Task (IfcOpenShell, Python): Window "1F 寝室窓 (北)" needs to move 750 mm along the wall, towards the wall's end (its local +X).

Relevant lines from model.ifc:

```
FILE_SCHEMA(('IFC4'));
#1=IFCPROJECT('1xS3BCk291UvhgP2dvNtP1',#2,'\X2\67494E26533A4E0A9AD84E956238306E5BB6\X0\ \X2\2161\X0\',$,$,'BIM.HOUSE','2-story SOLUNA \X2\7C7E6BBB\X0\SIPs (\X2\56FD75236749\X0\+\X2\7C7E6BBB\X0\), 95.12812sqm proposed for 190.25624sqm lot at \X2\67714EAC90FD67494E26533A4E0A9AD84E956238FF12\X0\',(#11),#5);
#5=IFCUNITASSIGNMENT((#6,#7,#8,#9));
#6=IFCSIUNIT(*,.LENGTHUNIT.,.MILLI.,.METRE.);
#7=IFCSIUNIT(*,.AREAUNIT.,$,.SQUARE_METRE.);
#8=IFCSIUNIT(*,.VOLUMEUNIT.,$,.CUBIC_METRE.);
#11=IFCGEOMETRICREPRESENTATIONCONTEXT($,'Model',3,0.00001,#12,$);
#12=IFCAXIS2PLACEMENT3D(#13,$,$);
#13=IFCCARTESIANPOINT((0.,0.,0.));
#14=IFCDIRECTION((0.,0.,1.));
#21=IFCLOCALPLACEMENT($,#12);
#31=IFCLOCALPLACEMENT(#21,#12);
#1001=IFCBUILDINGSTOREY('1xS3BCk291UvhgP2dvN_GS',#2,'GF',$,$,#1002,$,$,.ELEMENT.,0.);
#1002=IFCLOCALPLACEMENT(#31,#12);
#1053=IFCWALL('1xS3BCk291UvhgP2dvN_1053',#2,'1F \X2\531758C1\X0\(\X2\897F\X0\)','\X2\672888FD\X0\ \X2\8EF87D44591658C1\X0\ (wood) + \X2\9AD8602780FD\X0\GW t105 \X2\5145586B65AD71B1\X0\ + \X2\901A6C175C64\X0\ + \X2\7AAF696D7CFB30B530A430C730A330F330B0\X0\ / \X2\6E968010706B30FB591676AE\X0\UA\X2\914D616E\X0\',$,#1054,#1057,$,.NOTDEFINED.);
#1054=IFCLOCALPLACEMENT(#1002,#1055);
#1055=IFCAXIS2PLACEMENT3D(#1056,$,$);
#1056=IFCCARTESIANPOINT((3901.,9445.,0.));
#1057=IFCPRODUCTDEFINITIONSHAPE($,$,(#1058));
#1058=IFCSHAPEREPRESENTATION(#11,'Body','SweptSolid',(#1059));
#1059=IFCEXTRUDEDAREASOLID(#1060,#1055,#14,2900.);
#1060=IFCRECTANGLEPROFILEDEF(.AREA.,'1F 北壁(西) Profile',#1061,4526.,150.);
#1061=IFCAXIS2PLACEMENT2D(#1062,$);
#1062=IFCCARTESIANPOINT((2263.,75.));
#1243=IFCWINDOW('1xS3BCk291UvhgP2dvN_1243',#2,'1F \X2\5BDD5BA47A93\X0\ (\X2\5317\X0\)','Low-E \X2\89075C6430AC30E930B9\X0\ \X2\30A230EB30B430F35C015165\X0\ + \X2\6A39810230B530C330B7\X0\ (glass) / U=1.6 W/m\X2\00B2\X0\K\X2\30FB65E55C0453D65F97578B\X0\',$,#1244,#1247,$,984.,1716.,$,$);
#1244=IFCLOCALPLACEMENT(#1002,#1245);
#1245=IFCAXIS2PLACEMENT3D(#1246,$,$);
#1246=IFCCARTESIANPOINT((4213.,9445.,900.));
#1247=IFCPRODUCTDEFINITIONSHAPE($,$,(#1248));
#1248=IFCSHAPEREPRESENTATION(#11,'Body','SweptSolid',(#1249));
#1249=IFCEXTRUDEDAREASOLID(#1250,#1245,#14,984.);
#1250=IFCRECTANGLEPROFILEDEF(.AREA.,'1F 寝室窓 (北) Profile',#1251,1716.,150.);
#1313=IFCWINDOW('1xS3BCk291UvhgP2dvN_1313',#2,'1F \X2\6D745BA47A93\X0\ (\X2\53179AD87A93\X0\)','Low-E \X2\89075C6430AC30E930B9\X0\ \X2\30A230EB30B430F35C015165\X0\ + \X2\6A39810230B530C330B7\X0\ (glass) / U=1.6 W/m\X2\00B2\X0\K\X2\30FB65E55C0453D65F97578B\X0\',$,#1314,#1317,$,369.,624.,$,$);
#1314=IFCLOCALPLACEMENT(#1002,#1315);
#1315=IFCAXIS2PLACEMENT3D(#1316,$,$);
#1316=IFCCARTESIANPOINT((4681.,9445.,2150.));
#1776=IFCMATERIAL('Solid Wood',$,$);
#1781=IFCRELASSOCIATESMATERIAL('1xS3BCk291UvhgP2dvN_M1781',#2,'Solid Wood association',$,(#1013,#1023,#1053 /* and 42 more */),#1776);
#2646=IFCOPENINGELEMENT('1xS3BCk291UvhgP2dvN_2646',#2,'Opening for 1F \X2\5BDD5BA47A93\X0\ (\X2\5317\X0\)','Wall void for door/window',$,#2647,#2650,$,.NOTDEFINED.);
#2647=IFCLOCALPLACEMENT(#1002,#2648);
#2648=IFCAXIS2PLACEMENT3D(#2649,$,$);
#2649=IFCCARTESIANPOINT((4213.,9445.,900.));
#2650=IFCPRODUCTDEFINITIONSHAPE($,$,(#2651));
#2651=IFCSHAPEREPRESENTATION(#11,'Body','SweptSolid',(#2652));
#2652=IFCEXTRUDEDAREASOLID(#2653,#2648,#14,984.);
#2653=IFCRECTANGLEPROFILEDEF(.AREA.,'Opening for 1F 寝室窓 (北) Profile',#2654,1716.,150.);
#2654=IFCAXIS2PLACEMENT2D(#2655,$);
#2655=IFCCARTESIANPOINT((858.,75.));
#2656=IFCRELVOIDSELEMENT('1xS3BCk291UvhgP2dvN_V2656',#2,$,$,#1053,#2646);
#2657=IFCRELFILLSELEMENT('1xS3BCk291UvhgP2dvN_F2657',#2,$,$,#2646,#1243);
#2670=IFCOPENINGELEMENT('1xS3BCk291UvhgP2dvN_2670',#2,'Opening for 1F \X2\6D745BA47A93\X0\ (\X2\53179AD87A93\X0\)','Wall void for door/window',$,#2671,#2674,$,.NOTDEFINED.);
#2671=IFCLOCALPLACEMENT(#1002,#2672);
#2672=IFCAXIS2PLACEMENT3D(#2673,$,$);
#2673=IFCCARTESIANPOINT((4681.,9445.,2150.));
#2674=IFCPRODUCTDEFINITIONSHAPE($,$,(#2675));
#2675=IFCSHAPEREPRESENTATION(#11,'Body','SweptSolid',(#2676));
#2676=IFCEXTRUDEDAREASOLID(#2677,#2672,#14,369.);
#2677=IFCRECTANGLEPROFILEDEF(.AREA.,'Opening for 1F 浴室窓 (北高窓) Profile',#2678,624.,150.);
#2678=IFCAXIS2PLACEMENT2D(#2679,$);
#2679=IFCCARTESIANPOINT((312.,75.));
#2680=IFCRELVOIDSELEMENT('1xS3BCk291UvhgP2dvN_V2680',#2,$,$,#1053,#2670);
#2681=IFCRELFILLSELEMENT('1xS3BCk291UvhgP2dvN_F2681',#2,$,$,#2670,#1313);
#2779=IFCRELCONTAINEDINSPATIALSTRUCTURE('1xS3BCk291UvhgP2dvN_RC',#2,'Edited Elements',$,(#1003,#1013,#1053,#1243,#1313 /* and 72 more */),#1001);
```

```python
import ifcopenshell
import ifcopenshell.api.geometry
import ifcopenshell.util.placement
import ifcopenshell.util.unit

model = ifcopenshell.open("model.ifc")
unit_scale = ifcopenshell.util.unit.calculate_unit_scale(model)

window = model.by_guid("1xS3BCk291UvhgP2dvN_1243")
opening = window.FillsVoids[0].RelatingOpeningElement
wall = opening.VoidsElements[0].RelatingBuildingElement

wall_matrix = ifcopenshell.util.placement.get_local_placement(wall.ObjectPlacement)
shift = wall_matrix[:3, 0] * 0.75 / unit_scale
before = ifcopenshell.util.placement.get_local_placement(window.ObjectPlacement)[:3, 3].copy()

# The window is not placed relative to its opening, so move both.
for product in (opening, window):
    matrix = ifcopenshell.util.placement.get_local_placement(product.ObjectPlacement)
    matrix[:3, 3] += shift
    ifcopenshell.api.geometry.edit_object_placement(model, product=product, matrix=matrix, is_si=False)

after = ifcopenshell.util.placement.get_local_placement(window.ObjectPlacement)[:3, 3]
print("window moved by", (after - before).round(3) + 0.0)

model.write("model_edited.ifc")
```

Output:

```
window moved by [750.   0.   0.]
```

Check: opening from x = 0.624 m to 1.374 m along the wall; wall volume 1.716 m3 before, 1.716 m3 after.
